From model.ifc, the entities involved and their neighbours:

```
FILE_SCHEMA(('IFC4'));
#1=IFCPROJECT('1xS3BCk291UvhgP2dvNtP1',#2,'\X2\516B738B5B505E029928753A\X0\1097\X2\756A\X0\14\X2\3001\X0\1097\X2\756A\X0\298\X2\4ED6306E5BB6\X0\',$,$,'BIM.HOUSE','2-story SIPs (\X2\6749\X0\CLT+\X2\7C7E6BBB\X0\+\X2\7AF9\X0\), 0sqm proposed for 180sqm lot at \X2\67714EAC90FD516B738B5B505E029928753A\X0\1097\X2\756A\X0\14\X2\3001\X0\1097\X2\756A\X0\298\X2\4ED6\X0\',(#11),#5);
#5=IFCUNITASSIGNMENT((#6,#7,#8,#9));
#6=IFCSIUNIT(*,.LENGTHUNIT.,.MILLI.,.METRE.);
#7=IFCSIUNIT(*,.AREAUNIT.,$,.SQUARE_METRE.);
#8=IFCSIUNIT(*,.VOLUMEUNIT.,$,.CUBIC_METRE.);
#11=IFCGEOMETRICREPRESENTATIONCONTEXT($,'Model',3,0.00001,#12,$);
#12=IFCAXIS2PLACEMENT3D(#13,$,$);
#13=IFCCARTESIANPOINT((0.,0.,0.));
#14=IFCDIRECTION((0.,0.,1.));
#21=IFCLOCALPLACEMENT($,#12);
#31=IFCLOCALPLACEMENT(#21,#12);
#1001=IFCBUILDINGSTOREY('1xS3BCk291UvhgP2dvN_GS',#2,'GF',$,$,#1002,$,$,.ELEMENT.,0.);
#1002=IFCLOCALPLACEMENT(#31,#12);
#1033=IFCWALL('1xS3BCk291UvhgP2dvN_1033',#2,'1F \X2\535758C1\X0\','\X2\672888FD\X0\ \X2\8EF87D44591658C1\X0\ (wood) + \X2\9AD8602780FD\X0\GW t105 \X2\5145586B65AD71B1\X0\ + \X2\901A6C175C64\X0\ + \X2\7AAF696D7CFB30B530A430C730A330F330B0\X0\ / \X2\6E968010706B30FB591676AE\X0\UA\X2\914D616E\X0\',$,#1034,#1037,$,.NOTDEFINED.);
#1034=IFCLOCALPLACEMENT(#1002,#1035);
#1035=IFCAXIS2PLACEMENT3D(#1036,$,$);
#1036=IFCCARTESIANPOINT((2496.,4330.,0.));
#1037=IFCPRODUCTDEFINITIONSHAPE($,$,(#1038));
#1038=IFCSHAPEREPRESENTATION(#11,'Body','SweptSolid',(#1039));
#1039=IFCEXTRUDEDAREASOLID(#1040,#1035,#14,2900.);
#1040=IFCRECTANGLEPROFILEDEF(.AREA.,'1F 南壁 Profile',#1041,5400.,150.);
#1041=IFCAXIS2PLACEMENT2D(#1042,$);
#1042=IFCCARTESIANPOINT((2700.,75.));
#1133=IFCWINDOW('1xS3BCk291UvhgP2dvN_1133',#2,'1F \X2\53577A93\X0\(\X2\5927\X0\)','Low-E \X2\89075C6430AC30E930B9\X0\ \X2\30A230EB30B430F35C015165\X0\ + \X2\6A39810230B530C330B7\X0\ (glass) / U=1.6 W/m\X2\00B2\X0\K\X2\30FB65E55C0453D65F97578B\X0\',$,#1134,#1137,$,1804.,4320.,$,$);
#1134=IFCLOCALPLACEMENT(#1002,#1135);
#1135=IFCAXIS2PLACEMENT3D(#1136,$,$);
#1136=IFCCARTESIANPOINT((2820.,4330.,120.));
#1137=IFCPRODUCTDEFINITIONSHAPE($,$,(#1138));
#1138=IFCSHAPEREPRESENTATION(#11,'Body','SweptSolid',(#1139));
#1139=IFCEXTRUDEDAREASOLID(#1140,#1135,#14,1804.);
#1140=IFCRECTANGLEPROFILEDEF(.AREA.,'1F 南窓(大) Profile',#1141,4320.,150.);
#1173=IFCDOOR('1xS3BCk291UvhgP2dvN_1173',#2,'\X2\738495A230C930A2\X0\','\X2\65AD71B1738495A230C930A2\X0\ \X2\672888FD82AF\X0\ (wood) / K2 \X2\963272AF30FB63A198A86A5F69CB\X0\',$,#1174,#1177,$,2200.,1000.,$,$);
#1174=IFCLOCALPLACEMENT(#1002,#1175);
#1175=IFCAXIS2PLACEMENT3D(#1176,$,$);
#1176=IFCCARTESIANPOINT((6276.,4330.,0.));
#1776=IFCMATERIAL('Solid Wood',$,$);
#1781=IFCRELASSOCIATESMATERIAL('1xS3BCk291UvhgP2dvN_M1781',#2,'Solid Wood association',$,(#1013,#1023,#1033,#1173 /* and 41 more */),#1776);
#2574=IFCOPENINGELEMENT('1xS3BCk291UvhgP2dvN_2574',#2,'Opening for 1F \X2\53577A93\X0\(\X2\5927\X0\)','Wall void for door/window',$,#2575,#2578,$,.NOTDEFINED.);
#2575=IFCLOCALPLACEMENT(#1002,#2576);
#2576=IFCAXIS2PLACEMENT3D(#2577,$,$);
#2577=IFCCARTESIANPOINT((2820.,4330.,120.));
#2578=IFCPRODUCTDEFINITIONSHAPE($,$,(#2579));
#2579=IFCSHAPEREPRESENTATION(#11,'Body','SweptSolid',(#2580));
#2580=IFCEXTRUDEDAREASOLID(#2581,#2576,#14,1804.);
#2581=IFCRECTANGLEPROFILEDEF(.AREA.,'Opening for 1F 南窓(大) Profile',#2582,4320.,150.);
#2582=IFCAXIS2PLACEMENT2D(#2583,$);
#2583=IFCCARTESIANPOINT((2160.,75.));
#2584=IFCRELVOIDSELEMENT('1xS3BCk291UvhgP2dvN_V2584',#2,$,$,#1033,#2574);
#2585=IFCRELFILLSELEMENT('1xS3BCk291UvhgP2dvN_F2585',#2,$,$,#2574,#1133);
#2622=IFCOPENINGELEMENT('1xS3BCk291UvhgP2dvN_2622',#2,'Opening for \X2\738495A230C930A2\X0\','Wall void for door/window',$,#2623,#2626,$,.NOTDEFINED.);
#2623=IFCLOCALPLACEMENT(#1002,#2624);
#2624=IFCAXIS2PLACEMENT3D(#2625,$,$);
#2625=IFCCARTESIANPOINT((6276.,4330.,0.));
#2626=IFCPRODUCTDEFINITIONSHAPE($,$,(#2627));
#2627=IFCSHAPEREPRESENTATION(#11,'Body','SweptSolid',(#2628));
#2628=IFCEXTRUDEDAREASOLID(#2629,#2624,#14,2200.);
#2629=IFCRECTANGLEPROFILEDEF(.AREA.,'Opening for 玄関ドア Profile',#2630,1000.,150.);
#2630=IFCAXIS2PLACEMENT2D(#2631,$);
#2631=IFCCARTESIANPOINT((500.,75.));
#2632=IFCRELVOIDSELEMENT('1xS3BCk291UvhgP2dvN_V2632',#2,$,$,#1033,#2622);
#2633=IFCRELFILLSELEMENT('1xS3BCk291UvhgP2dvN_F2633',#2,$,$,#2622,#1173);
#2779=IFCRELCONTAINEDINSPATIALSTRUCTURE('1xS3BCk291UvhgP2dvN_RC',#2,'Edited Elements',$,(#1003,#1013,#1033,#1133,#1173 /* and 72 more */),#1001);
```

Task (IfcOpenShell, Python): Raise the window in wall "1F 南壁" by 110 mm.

```python
import numpy as np
import ifcopenshell
import ifcopenshell.api.geometry
import ifcopenshell.util.placement
import ifcopenshell.util.unit

model = ifcopenshell.open("model.ifc")
unit_scale = ifcopenshell.util.unit.calculate_unit_scale(model)

window = model.by_guid("1xS3BCk291UvhgP2dvN_1133")
opening = window.FillsVoids[0].RelatingOpeningElement
dz = 110.0

shift = np.array([0.0, 0.0, dz])
# The window is not placed relative to its opening, so move both.
for product in (opening, window):
    matrix = ifcopenshell.util.placement.get_local_placement(product.ObjectPlacement)
    matrix[:3, 3] += shift
    ifcopenshell.api.geometry.edit_object_placement(model, product=product, matrix=matrix, is_si=False)

print(f"moved by {dz * unit_scale:+.3f} m")

model.write("model_edited.ifc")
```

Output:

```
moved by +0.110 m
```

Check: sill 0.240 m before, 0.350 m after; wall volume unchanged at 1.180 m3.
